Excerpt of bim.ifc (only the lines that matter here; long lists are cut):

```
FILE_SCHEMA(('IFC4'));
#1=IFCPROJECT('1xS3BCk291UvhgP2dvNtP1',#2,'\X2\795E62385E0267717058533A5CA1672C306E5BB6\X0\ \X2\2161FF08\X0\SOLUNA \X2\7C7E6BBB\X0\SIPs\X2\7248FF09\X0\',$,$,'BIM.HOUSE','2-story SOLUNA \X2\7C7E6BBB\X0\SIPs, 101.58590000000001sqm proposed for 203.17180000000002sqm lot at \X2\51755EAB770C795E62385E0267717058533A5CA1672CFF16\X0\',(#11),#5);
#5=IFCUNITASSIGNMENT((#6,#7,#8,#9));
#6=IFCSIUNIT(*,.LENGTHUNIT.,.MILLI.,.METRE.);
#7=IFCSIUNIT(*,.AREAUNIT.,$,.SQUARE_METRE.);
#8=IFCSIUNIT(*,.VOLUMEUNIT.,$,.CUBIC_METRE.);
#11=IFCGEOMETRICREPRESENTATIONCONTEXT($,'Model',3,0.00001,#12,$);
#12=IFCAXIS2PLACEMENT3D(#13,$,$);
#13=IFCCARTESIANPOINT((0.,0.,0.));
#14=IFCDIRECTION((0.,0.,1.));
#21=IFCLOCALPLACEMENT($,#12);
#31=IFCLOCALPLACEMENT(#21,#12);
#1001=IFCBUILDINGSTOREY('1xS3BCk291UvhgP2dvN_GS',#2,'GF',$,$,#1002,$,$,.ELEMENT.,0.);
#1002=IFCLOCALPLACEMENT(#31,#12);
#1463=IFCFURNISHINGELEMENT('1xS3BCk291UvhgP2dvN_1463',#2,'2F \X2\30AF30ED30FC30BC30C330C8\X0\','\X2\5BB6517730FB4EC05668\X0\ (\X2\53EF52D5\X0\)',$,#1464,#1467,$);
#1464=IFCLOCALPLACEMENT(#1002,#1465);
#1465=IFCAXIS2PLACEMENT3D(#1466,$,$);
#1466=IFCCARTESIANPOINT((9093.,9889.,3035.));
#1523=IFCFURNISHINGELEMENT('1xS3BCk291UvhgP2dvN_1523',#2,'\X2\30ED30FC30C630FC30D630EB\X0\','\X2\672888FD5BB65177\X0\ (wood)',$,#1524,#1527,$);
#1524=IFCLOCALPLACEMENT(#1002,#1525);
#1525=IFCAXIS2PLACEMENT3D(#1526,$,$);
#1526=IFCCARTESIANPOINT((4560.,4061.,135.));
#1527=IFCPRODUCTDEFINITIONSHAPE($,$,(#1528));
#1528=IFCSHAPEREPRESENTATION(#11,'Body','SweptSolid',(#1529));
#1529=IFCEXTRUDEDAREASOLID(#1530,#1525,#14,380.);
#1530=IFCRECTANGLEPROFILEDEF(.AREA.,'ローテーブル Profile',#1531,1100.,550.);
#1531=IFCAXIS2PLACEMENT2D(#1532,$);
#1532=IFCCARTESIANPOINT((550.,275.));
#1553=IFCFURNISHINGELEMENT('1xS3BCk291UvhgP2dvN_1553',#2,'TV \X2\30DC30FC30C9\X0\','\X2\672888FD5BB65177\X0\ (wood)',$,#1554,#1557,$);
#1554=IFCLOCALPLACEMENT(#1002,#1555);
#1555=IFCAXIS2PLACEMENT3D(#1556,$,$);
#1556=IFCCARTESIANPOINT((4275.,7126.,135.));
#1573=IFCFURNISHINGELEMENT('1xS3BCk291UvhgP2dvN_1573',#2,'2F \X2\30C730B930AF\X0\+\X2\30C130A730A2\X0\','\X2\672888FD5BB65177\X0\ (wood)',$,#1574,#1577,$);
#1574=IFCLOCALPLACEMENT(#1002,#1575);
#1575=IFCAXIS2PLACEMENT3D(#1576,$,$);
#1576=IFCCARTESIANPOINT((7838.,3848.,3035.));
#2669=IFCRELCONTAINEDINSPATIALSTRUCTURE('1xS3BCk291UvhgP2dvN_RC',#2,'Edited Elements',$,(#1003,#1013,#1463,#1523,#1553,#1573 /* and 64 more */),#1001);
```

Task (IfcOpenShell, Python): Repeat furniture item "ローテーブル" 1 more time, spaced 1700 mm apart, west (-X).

```python
import numpy as np
import ifcopenshell
import ifcopenshell.api.geometry
import ifcopenshell.api.root
import ifcopenshell.util.element
import ifcopenshell.util.placement
import ifcopenshell.util.unit

model = ifcopenshell.open("bim.ifc")
unit_scale = ifcopenshell.util.unit.calculate_unit_scale(model)


def reuse_history(source, copy):
    """copy_class also copies each property set's owner history, people and application; keep the originals."""
    for rel in copy.IsDefinedBy:
        if rel.is_a("IfcRelDefinesByProperties") and (history := rel.RelatingPropertyDefinition.OwnerHistory):
            rel.RelatingPropertyDefinition.OwnerHistory = source.OwnerHistory
            ifcopenshell.util.element.remove_deep2(model, history)


source = model.by_id(1523)
base = ifcopenshell.util.placement.get_local_placement(source.ObjectPlacement)
step = np.array([-1.0, 0.0, 0.0]) * 1.7 / unit_scale

for i in range(1, 2):
    copy = ifcopenshell.api.root.copy_class(model, product=source)
    copy.Representation = ifcopenshell.util.element.copy_deep(
        model, source.Representation, exclude=["IfcGeometricRepresentationContext", "IfcRepresentationMap"]
    )
    reuse_history(source, copy)
    matrix = base.copy()
    matrix[:3, 3] += i * step
    print("added at", matrix[:3, 3].round(3) + 0.0)
    ifcopenshell.api.geometry.edit_object_placement(model, product=copy, matrix=matrix, is_si=False)

model.write("bim_edited.ifc")
```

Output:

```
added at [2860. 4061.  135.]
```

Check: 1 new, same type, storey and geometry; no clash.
